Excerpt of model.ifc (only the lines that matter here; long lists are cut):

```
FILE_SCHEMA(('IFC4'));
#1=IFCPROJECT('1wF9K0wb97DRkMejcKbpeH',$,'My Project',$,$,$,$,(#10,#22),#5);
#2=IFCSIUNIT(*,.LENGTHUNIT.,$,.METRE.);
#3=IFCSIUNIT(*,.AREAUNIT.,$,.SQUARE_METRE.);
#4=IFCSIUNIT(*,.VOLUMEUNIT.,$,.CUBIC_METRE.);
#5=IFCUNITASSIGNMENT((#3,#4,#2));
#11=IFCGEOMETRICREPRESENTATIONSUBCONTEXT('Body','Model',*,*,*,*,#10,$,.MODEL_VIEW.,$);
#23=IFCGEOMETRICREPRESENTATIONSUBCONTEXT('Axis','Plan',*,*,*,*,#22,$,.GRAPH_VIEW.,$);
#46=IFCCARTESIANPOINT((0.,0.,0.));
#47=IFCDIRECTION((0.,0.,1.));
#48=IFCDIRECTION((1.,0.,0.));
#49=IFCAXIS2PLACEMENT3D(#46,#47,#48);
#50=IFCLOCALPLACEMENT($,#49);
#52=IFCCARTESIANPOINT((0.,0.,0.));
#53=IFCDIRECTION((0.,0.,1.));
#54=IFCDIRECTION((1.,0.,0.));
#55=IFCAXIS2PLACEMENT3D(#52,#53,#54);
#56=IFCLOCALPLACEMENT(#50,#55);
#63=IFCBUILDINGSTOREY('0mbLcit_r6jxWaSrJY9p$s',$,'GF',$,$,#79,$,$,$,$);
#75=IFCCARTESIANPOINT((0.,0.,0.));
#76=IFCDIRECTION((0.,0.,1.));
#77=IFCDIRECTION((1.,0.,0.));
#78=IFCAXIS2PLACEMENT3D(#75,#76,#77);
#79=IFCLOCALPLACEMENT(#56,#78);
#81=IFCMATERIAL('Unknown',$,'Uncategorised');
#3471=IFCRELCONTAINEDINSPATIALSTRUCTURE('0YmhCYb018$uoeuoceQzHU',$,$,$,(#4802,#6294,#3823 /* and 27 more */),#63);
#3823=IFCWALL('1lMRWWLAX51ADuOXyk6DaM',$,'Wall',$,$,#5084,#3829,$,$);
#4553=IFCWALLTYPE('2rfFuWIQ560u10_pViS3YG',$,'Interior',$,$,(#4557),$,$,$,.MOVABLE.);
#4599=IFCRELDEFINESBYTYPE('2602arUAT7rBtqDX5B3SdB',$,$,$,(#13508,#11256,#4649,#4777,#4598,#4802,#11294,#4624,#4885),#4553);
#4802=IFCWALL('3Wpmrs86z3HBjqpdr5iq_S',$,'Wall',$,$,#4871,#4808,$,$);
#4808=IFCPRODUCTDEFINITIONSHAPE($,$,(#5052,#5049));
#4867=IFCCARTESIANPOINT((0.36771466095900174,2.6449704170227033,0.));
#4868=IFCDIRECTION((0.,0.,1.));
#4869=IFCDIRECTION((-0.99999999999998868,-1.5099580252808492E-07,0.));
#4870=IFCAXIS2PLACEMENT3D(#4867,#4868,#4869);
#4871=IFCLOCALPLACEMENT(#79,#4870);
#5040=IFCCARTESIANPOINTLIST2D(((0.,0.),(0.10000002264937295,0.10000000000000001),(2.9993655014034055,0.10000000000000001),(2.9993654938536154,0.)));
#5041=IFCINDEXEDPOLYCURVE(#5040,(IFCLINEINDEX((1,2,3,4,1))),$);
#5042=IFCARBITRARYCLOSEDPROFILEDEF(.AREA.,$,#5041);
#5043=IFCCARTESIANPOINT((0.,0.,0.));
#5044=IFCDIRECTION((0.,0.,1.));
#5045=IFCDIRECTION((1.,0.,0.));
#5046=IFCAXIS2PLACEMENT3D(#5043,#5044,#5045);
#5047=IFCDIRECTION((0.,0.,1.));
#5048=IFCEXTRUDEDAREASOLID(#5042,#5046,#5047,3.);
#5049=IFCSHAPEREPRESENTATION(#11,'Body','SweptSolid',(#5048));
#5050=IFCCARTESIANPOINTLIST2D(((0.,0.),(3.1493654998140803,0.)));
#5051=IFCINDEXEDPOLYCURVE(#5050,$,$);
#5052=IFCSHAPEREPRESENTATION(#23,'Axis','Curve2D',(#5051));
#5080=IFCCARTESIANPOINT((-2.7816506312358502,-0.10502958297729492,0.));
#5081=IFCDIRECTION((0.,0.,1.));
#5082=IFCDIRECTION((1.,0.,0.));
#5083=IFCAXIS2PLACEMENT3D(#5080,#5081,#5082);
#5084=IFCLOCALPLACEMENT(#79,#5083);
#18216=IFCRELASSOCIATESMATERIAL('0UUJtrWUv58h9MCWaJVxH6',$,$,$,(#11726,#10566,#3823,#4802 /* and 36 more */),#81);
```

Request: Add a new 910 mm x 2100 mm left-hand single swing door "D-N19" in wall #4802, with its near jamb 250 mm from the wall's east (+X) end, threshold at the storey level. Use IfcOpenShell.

```python
import numpy as np
import ifcopenshell
import ifcopenshell.api.feature
import ifcopenshell.api.geometry
import ifcopenshell.api.root
import ifcopenshell.api.spatial
import ifcopenshell.geom
import ifcopenshell.util.element
import ifcopenshell.util.placement
import ifcopenshell.util.representation
import ifcopenshell.util.shape
import ifcopenshell.util.unit

model = ifcopenshell.open("model.ifc")
unit_scale = ifcopenshell.util.unit.calculate_unit_scale(model)
settings = ifcopenshell.geom.settings()


def volume(element):
    """Net volume in cubic metres, openings subtracted."""
    shape = ifcopenshell.geom.create_shape(settings, element)
    return ifcopenshell.util.shape.get_volume(shape.geometry)


wall = model.by_guid("3Wpmrs86z3HBjqpdr5iq_S")
storey = ifcopenshell.util.element.get_container(wall, ifc_class="IfcBuildingStorey")
context = ifcopenshell.util.representation.get_context(model, "Model", "Body", "MODEL_VIEW")
before = volume(wall)

width, height, from_end, sill = 0.91, 2.1, 0.25, 0.0  # metres

# The wall runs along its own X axis, and the end named is its -X end.
wall_shape = ifcopenshell.geom.create_shape(settings, wall)
x, y, z = ifcopenshell.util.shape.get_vertices(wall_shape.geometry).T
start = x.min() + from_end
face, thickness = float(y.min()), float(y.max() - y.min())
wall_matrix = ifcopenshell.util.placement.get_local_placement(wall.ObjectPlacement)
level = ifcopenshell.util.placement.get_local_placement(storey.ObjectPlacement)[2, 3]


def in_wall(x, y):
    """Placement at x, y metres in the wall's axes, at sill height."""
    matrix = wall_matrix.copy()
    matrix[:, 3] = wall_matrix @ np.array([x / unit_scale, y / unit_scale, 0.0, 1.0])
    matrix[2, 3] = level + sill / unit_scale
    return matrix


# Opening: a box that overshoots both wall faces by 50 mm.
opening = ifcopenshell.api.root.create_entity(model, ifc_class="IfcOpeningElement", predefined_type="OPENING")
box = ifcopenshell.api.geometry.add_wall_representation(
    model, context=context, length=width, height=height, thickness=thickness + 0.1
)
ifcopenshell.api.geometry.assign_representation(model, product=opening, representation=box)
ifcopenshell.api.geometry.edit_object_placement(model, product=opening, matrix=in_wall(start, face - 0.05), is_si=False)
ifcopenshell.api.feature.add_feature(model, feature=opening, element=wall)

door = ifcopenshell.api.root.create_entity(model, ifc_class="IfcDoor", name="D-N19", predefined_type="DOOR")
door.OverallWidth, door.OverallHeight = width / unit_scale, height / unit_scale
door.OperationType = "SINGLE_SWING_LEFT"
body = ifcopenshell.api.geometry.add_door_representation(
    model,
    context=context,
    overall_width=door.OverallWidth,
    overall_height=door.OverallHeight,
    operation_type="SINGLE_SWING_LEFT",
    lining_properties={"LiningDepth": thickness / unit_scale, "ThresholdDepth": thickness / unit_scale},
)
ifcopenshell.api.geometry.assign_representation(model, product=door, representation=body)
ifcopenshell.api.spatial.assign_container(model, products=[door], relating_structure=storey)
ifcopenshell.api.feature.add_filling(model, opening=opening, element=door)

# The lining spans the wall, so the door starts at the wall face.
ifcopenshell.api.geometry.edit_object_placement(model, product=door, matrix=in_wall(start, face), is_si=False)

after = volume(wall)

print(f"wall volume {before:.3f} -> {after:.3f} m3")

model.write("model_edited.ifc")
```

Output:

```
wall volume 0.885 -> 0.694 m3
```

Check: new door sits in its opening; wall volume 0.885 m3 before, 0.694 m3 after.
